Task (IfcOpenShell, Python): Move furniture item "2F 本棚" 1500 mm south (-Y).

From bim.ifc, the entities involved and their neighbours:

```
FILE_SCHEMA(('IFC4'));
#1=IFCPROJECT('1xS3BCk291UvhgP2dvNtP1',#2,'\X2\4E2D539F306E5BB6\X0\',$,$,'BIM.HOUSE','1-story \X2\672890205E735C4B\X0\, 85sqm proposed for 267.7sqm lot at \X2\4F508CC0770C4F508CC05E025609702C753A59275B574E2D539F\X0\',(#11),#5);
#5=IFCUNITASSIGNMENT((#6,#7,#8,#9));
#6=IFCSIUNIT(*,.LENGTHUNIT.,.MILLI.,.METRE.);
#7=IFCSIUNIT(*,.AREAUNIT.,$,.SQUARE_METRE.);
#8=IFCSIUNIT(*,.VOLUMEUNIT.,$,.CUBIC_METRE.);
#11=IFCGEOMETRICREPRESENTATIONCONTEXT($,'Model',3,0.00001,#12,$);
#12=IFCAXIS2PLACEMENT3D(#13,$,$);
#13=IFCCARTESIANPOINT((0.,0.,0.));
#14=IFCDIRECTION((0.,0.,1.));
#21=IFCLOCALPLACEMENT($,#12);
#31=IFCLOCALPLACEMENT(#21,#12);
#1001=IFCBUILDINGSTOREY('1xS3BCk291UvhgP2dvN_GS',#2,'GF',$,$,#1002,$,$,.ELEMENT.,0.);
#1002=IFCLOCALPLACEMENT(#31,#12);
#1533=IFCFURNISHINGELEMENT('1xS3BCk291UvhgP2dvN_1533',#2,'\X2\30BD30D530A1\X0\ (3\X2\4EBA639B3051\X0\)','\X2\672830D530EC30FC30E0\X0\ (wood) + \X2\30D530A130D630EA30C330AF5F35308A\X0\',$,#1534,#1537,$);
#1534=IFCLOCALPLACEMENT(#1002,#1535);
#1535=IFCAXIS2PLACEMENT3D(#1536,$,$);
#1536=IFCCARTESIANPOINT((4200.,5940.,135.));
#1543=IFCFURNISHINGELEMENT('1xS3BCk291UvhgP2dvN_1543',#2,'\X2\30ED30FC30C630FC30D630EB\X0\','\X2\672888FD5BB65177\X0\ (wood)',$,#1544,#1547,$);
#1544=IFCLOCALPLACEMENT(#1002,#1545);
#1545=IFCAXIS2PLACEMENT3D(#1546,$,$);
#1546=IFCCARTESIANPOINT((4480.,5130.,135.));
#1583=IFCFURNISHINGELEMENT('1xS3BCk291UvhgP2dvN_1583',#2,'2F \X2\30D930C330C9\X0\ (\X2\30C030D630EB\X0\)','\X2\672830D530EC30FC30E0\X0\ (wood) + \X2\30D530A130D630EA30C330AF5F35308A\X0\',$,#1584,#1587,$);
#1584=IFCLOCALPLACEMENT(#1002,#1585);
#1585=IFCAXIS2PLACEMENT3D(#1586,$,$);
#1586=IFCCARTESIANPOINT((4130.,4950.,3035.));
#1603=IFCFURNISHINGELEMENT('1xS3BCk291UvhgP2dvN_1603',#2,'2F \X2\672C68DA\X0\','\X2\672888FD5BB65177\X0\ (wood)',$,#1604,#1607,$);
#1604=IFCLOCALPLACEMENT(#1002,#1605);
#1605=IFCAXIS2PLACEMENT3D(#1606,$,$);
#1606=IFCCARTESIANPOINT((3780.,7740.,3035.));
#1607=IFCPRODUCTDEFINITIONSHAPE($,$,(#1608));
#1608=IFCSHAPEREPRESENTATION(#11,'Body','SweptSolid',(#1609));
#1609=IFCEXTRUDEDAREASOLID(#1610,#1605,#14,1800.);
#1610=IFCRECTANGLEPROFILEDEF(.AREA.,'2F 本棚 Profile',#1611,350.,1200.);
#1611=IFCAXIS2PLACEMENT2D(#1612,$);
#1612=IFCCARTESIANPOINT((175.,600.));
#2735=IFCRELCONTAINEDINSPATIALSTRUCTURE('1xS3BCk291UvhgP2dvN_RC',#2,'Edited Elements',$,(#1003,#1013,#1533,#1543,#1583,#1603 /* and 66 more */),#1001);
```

```python
import ifcopenshell
import ifcopenshell.api.geometry
import ifcopenshell.util.placement
import ifcopenshell.util.unit

model = ifcopenshell.open("bim.ifc")
unit_scale = ifcopenshell.util.unit.calculate_unit_scale(model)

item = model.by_guid("1xS3BCk291UvhgP2dvN_1603")
matrix = ifcopenshell.util.placement.get_local_placement(item.ObjectPlacement)
matrix[1, 3] -= 1.5 / unit_scale
ifcopenshell.api.geometry.edit_object_placement(model, product=item, matrix=matrix, is_si=False)

print(ifcopenshell.util.placement.get_local_placement(item.ObjectPlacement).round(3) + 0.0)

model.write("bim_edited.ifc")
```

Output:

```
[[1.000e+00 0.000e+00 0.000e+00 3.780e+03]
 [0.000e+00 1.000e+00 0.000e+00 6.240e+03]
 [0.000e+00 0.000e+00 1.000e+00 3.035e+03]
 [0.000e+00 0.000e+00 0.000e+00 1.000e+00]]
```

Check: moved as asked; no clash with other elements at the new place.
